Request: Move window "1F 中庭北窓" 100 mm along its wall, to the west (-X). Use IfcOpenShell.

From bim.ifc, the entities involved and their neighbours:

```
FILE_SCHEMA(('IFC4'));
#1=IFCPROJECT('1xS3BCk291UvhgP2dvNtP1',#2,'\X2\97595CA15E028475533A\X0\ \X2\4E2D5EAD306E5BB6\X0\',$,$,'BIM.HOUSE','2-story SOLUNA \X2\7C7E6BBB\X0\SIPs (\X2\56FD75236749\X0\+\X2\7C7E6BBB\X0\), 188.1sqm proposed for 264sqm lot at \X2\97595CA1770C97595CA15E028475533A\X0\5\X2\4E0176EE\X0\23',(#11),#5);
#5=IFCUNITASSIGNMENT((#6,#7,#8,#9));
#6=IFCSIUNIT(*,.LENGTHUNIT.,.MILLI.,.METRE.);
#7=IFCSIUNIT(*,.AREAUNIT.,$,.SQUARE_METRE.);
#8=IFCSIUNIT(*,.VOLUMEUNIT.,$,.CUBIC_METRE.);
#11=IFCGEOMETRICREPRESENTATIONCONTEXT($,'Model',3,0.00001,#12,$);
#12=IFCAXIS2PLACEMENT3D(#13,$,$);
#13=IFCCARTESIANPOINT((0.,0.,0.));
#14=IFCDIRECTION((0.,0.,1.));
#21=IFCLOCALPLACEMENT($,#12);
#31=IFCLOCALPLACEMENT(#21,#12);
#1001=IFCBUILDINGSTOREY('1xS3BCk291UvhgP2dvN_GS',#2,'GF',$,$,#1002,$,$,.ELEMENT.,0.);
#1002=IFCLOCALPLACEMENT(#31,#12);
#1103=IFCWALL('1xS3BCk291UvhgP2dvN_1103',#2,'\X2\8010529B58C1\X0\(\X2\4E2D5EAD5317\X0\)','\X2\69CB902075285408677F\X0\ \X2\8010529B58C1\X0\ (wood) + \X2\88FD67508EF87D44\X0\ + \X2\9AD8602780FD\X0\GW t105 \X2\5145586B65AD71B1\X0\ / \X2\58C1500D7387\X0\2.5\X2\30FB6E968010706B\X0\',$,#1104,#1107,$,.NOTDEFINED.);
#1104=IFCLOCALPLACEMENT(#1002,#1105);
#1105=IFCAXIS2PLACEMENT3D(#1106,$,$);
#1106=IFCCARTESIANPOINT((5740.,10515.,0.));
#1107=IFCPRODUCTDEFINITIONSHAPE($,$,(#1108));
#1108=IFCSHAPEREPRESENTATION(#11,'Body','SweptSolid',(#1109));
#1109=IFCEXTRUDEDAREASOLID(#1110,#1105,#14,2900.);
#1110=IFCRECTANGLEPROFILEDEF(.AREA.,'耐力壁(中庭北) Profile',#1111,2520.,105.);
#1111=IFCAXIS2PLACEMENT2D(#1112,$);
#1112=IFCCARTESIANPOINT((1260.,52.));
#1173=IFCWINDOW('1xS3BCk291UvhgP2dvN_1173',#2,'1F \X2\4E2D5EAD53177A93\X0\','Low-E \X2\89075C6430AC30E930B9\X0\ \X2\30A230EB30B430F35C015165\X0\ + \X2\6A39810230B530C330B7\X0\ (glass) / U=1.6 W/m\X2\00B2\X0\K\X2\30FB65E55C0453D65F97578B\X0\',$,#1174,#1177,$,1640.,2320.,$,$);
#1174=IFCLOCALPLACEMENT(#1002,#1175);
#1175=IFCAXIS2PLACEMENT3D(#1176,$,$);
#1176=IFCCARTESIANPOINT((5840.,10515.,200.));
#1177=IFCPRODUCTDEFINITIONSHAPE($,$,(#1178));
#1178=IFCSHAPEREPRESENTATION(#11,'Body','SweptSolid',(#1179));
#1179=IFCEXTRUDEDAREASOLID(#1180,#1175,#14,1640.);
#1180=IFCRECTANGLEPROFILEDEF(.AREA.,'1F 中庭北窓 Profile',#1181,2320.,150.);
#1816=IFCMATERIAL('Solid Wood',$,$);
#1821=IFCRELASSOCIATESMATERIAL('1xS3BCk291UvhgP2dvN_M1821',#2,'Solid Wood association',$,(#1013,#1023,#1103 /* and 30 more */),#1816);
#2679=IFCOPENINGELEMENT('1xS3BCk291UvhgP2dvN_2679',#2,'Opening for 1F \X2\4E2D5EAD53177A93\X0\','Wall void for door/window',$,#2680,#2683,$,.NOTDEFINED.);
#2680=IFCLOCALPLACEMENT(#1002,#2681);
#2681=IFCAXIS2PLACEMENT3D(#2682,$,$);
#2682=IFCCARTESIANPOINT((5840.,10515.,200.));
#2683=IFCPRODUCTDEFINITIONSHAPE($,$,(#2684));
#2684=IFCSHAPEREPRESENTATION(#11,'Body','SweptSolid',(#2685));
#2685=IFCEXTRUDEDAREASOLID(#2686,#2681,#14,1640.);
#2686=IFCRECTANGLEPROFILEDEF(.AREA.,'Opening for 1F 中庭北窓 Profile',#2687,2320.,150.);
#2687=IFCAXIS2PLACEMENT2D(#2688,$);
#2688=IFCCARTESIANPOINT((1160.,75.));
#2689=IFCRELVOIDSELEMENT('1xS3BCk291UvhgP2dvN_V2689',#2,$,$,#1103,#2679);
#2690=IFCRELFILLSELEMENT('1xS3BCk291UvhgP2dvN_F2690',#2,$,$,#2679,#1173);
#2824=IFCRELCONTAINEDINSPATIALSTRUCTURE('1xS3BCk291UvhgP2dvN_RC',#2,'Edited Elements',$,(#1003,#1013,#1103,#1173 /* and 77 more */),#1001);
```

```python
import ifcopenshell
import ifcopenshell.api.geometry
import ifcopenshell.util.placement
import ifcopenshell.util.unit

model = ifcopenshell.open("bim.ifc")
unit_scale = ifcopenshell.util.unit.calculate_unit_scale(model)

window = model.by_guid("1xS3BCk291UvhgP2dvN_1173")
opening = window.FillsVoids[0].RelatingOpeningElement
wall = opening.VoidsElements[0].RelatingBuildingElement

wall_matrix = ifcopenshell.util.placement.get_local_placement(wall.ObjectPlacement)
shift = wall_matrix[:3, 0] * -0.1 / unit_scale
before = ifcopenshell.util.placement.get_local_placement(window.ObjectPlacement)[:3, 3].copy()

# The window is not placed relative to its opening, so move both.
for product in (opening, window):
    matrix = ifcopenshell.util.placement.get_local_placement(product.ObjectPlacement)
    matrix[:3, 3] += shift
    ifcopenshell.api.geometry.edit_object_placement(model, product=product, matrix=matrix, is_si=False)

after = ifcopenshell.util.placement.get_local_placement(window.ObjectPlacement)[:3, 3]
print("window moved by", (after - before).round(3) + 0.0)

model.write("bim_updated.ifc")
```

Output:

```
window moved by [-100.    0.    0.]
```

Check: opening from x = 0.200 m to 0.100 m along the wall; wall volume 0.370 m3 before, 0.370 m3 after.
